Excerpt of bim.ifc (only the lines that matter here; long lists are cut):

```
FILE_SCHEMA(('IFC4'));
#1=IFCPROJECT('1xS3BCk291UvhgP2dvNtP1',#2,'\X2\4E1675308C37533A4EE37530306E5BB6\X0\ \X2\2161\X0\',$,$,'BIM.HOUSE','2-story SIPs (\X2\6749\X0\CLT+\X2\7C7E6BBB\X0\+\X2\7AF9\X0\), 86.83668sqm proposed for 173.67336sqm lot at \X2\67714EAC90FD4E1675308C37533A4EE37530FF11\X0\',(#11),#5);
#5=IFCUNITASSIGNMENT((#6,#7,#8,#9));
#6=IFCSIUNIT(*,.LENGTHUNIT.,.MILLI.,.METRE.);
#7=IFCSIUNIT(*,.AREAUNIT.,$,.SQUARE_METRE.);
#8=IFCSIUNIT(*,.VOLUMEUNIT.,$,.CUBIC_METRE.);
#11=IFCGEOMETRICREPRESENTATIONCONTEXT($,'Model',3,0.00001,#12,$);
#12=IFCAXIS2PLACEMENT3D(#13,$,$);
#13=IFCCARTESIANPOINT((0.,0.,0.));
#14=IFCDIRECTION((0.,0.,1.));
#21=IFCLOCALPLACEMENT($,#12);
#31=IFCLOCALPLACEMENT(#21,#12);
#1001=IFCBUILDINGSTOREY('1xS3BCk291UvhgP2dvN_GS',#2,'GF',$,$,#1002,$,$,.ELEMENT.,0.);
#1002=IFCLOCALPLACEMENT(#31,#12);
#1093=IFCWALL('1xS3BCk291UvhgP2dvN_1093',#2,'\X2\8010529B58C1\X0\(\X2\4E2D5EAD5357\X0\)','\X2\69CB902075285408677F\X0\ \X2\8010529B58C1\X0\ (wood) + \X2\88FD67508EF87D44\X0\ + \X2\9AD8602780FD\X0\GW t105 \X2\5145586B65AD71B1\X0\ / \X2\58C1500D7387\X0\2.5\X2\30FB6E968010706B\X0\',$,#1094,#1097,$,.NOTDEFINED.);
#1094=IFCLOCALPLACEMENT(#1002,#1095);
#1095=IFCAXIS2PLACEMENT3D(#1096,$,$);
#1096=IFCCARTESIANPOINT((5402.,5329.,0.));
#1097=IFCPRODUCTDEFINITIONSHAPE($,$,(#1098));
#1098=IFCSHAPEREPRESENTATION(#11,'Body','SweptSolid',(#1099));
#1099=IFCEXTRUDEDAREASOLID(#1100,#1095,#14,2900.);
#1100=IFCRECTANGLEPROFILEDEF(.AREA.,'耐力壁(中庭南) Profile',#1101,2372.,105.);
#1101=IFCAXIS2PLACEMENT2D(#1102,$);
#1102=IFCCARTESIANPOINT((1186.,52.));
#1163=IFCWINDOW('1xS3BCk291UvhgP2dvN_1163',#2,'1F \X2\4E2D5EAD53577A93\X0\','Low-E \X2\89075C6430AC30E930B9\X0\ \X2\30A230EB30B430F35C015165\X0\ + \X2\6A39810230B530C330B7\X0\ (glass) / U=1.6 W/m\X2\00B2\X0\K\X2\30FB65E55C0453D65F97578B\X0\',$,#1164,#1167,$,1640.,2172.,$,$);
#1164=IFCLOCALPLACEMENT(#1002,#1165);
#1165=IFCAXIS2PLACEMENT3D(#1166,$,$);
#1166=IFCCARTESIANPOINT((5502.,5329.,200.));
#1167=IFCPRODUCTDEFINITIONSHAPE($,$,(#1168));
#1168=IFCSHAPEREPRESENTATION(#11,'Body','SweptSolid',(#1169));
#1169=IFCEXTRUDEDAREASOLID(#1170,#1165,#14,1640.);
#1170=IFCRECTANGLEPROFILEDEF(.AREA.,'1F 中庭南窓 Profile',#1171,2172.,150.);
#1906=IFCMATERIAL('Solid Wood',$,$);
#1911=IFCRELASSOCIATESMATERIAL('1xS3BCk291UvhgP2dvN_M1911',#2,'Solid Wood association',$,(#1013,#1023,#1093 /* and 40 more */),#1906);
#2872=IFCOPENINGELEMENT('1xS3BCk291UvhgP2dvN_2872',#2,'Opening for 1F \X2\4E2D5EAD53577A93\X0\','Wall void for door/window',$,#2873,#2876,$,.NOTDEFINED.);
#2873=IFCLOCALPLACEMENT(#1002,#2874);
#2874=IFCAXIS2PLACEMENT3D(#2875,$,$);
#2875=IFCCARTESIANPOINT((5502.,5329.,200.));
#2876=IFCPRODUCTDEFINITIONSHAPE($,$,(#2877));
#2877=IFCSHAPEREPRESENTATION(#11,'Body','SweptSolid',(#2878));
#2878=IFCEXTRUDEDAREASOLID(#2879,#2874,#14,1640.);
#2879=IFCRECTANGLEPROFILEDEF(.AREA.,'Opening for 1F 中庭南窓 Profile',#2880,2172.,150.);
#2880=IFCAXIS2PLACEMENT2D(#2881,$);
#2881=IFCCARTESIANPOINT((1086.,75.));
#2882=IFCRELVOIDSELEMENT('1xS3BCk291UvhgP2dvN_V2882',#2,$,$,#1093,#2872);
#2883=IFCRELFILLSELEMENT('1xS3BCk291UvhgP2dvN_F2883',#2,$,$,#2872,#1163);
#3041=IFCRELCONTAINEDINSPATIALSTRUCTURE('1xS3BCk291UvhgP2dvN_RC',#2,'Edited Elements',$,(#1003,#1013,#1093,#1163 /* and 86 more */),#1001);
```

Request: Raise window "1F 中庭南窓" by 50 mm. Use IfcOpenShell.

```python
import numpy as np
import ifcopenshell
import ifcopenshell.api.geometry
import ifcopenshell.util.placement
import ifcopenshell.util.unit

model = ifcopenshell.open("bim.ifc")
unit_scale = ifcopenshell.util.unit.calculate_unit_scale(model)

window = model.by_guid("1xS3BCk291UvhgP2dvN_1163")
opening = window.FillsVoids[0].RelatingOpeningElement
dz = 50.0

shift = np.array([0.0, 0.0, dz])
# The window is not placed relative to its opening, so move both.
for product in (opening, window):
    matrix = ifcopenshell.util.placement.get_local_placement(product.ObjectPlacement)
    matrix[:3, 3] += shift
    ifcopenshell.api.geometry.edit_object_placement(model, product=product, matrix=matrix, is_si=False)

print(f"moved by {dz * unit_scale:+.3f} m")

model.write("bim_rev.ifc")
```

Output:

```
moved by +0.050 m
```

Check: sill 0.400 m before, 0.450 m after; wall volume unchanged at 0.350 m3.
